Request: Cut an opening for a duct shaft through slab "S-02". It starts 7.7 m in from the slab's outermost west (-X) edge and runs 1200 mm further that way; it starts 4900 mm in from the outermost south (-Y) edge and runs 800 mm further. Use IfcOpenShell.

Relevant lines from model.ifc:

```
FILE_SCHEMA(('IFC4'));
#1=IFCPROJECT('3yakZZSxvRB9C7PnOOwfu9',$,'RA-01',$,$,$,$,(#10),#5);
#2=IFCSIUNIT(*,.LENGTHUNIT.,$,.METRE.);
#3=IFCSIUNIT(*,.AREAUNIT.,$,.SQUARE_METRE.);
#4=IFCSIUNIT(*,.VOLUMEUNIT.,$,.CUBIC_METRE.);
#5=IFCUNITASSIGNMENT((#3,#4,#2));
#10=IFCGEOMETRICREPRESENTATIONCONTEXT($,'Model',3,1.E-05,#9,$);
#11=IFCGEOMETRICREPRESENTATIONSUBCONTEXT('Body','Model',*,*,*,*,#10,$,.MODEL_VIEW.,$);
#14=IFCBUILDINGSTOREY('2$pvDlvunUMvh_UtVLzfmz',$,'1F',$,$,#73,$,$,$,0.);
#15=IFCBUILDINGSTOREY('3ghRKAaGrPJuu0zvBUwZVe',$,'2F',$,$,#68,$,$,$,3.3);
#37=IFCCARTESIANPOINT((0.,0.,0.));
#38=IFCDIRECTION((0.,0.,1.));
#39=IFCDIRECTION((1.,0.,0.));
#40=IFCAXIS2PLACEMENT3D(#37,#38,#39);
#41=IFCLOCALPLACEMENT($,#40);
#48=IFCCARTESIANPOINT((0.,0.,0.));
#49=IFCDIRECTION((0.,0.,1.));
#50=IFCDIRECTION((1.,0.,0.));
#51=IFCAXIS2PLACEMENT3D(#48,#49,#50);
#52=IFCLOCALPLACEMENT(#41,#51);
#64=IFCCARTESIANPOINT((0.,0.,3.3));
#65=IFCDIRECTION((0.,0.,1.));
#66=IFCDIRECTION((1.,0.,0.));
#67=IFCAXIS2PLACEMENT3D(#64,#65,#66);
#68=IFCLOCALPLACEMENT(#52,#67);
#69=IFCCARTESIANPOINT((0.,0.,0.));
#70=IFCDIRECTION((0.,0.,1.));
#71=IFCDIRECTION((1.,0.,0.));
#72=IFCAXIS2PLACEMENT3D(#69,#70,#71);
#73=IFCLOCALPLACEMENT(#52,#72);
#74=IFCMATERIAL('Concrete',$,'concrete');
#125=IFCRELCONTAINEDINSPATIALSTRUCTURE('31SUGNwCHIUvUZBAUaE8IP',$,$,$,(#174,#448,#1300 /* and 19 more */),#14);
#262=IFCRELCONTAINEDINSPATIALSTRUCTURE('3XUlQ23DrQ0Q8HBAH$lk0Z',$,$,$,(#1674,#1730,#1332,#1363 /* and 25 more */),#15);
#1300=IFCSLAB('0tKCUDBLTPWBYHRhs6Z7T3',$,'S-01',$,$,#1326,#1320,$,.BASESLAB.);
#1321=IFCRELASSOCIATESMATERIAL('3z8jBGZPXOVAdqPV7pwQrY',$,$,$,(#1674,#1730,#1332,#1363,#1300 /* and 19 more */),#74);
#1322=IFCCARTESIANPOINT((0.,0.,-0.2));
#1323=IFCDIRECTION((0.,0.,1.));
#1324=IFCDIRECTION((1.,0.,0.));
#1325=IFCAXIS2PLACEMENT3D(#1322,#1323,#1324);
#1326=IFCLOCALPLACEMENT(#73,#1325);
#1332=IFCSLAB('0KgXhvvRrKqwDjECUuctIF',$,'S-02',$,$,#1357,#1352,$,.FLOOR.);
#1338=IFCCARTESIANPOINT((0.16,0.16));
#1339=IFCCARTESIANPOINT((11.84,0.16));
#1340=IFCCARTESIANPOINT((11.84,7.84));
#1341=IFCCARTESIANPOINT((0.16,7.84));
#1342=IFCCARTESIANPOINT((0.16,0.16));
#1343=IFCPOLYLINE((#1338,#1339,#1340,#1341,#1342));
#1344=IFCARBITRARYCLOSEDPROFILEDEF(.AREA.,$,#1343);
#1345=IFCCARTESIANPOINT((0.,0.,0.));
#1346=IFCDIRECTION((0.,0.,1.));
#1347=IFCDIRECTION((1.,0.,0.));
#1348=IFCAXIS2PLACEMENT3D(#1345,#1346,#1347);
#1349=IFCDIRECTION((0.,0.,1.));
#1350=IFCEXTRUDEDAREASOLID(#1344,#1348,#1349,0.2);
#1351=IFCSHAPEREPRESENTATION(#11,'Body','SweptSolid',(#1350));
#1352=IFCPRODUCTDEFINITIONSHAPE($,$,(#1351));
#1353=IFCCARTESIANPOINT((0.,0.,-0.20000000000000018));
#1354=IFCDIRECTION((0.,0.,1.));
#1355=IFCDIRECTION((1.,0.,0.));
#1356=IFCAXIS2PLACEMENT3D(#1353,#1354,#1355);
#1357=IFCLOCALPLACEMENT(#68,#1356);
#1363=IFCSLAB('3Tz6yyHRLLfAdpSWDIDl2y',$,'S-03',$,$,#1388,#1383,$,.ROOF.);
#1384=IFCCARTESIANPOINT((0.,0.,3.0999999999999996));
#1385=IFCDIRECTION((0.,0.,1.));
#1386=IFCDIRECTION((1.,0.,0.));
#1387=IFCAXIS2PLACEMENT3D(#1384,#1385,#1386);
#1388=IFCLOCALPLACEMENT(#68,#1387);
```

```python
import numpy as np
import ifcopenshell
import ifcopenshell.api.feature
import ifcopenshell.api.geometry
import ifcopenshell.api.root
import ifcopenshell.geom
import ifcopenshell.util.placement
import ifcopenshell.util.representation
import ifcopenshell.util.shape
import ifcopenshell.util.unit

model = ifcopenshell.open("model.ifc")
unit_scale = ifcopenshell.util.unit.calculate_unit_scale(model)
settings = ifcopenshell.geom.settings()


def volume(element):
    """Net volume in cubic metres, openings subtracted."""
    shape = ifcopenshell.geom.create_shape(settings, element)
    return ifcopenshell.util.shape.get_volume(shape.geometry)


slab = model.by_guid("0KgXhvvRrKqwDjECUuctIF")
before = volume(slab)

# Extent in the slab's own axes, in metres. The edges named are its -X and -Y sides.
slab_shape = ifcopenshell.geom.create_shape(settings, slab)
vertices = ifcopenshell.util.shape.get_vertices(slab_shape.geometry)
x_min, y_min, bottom = vertices.min(axis=0)
top = vertices[:, 2].max()

opening = ifcopenshell.api.root.create_entity(model, ifc_class="IfcOpeningElement", name="Duct shaft opening", predefined_type="OPENING")
context = ifcopenshell.util.representation.get_context(model, "Model", "Body", "MODEL_VIEW")
width, depth = 1.2, 0.8
outline = [(0.0, 0.0), (width, 0.0), (width, depth), (0.0, depth), (0.0, 0.0)]
# Overshoot both faces by 50 mm so the cut is clean.
shape = ifcopenshell.api.geometry.add_slab_representation(
    model, context=context, depth=top - bottom + 0.1, polyline=outline
)
ifcopenshell.api.geometry.assign_representation(model, product=opening, representation=shape)

matrix = ifcopenshell.util.placement.get_local_placement(slab.ObjectPlacement)
matrix[:, 3] = matrix @ np.append(np.array([x_min + 7.7, y_min + 4.9, bottom - 0.05]) / unit_scale, 1.0)
ifcopenshell.api.geometry.edit_object_placement(model, product=opening, matrix=matrix, is_si=False)
ifcopenshell.api.feature.add_feature(model, feature=opening, element=slab)

after = volume(slab)

print(f"slab volume {before:.3f} -> {after:.3f} m3")

model.write("model-out.ifc")
```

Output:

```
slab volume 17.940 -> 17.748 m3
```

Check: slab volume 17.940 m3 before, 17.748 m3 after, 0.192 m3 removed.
